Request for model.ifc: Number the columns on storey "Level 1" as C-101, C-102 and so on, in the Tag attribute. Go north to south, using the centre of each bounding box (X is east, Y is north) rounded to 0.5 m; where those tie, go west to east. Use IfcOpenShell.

First a look at what the model holds.

```python
import ifcopenshell
import ifcopenshell.util.element
import ifcopenshell.util.placement

model = ifcopenshell.open("model.ifc")
print(model.schema)
storey = next(s for s in model.by_type("IfcBuildingStorey") if s.Name == "Level 1")
columns = [e for e in ifcopenshell.util.element.get_decomposition(storey) if e.is_a("IfcColumn")]
for e in sorted(columns, key=lambda e: e.id()):
    origin = ifcopenshell.util.placement.get_local_placement(e.ObjectPlacement)[:3, 3]
    print(e.id(), e.Tag, e.Name, origin.round(2) + 0.0, sep=" | ")
```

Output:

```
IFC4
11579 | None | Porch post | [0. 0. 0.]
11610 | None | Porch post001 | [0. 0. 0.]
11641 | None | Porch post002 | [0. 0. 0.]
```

```python
import ifcopenshell
import ifcopenshell.geom
import ifcopenshell.util.element
import ifcopenshell.util.shape

model = ifcopenshell.open("model.ifc")
settings = ifcopenshell.geom.settings()
settings.set("use-world-coords", True)


def centre(element):
    shape = ifcopenshell.geom.create_shape(settings, element)
    return ifcopenshell.util.shape.get_bbox_centroid(shape.geometry)


storey = next(s for s in model.by_type("IfcBuildingStorey") if s.Name == "Level 1")
columns = [e for e in ifcopenshell.util.element.get_decomposition(storey) if e.is_a("IfcColumn")]

# Insertion points can sit at a corner or the storey origin, so sort by the geometry (in metres).
centres = {e: centre(e) for e in columns}
columns.sort(key=lambda e: (-round(centres[e][1] / 0.5), centres[e][0]))

for i, e in enumerate(columns, start=1):
    number = f"C-1{i:02d}"
    e.Tag = number
    print(e.id(), number)

model.write("model-out.ifc")
```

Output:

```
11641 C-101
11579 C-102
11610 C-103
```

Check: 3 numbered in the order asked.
